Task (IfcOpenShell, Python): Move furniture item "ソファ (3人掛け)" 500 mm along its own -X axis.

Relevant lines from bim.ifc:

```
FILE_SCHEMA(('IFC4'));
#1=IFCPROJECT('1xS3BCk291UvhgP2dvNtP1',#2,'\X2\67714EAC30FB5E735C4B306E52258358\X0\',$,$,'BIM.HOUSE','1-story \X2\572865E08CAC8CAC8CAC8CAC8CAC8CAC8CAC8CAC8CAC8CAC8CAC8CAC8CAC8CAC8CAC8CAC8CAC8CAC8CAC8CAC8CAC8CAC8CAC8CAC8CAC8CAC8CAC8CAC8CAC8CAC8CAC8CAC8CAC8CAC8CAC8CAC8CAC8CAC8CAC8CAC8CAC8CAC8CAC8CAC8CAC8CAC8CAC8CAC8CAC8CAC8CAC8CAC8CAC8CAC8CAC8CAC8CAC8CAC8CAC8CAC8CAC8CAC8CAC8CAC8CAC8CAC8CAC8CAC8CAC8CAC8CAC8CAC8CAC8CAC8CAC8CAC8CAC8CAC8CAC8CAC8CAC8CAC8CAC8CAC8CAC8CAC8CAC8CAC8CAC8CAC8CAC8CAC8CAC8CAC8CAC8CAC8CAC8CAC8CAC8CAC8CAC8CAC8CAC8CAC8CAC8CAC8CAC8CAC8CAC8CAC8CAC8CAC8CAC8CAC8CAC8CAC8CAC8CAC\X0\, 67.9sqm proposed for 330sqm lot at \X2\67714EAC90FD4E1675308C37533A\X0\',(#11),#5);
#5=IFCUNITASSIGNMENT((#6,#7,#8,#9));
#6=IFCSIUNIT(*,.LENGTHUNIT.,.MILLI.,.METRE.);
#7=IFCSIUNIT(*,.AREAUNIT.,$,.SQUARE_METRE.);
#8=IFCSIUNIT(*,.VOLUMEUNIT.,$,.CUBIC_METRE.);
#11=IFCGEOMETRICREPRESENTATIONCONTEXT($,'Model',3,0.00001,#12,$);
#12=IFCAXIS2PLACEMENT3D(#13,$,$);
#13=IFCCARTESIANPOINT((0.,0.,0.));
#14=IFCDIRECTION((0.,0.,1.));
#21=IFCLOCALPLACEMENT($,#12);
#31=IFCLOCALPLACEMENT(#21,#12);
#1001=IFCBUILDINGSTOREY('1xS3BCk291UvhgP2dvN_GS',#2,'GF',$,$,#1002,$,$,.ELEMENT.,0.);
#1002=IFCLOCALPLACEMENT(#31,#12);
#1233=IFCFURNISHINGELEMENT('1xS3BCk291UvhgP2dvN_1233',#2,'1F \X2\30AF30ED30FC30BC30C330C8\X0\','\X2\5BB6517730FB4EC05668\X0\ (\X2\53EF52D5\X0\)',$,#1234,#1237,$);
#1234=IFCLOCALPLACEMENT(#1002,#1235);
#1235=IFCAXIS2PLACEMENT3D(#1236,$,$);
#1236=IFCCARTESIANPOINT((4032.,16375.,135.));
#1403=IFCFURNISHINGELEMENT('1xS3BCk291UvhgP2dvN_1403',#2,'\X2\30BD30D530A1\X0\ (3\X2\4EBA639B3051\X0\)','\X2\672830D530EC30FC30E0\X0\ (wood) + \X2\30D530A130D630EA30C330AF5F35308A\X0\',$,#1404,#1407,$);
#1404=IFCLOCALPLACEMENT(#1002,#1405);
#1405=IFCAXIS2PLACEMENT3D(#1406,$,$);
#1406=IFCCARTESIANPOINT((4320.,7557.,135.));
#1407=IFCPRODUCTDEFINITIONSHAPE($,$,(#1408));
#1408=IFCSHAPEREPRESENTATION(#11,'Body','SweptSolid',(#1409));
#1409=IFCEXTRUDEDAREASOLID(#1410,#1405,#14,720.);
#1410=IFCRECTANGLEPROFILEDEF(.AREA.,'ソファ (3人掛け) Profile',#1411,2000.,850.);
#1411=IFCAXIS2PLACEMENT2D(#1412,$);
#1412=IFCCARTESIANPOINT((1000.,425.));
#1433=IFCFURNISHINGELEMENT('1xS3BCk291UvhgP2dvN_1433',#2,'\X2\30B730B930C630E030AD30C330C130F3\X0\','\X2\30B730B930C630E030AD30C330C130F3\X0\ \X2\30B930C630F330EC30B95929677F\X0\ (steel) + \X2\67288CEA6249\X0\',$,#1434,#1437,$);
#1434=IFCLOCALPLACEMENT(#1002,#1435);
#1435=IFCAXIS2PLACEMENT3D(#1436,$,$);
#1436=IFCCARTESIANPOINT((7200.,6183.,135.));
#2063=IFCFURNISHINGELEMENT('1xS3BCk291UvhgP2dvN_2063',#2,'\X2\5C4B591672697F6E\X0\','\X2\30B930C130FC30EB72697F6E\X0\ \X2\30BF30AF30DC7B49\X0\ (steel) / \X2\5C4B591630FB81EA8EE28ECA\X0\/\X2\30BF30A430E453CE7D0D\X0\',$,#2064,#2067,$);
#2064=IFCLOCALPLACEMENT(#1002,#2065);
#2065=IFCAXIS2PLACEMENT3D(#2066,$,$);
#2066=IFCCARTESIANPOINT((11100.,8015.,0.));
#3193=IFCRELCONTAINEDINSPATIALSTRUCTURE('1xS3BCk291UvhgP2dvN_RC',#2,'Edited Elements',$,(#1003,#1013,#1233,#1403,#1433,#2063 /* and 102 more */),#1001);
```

```python
import ifcopenshell
import ifcopenshell.api.geometry
import ifcopenshell.util.placement
import ifcopenshell.util.unit

model = ifcopenshell.open("bim.ifc")
unit_scale = ifcopenshell.util.unit.calculate_unit_scale(model)

item = model.by_guid("1xS3BCk291UvhgP2dvN_1403")
matrix = ifcopenshell.util.placement.get_local_placement(item.ObjectPlacement)
matrix[:3, 3] -= matrix[:3, 0] * 0.5 / unit_scale
ifcopenshell.api.geometry.edit_object_placement(model, product=item, matrix=matrix, is_si=False)

print(ifcopenshell.util.placement.get_local_placement(item.ObjectPlacement).round(3) + 0.0)

model.write("bim_updated.ifc")
```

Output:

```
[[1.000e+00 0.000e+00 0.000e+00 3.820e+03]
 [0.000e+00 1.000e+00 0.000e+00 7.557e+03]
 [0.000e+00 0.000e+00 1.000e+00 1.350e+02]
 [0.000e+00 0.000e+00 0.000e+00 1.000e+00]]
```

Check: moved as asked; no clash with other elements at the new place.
